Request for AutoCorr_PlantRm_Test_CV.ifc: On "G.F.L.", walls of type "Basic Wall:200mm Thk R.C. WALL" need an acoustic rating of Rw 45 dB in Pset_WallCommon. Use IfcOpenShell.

First a look at what the model holds.

```python
import ifcopenshell
import ifcopenshell.util.element

model = ifcopenshell.open("AutoCorr_PlantRm_Test_CV.ifc")
print(model.schema)
storey = next(s for s in model.by_type("IfcBuildingStorey") if s.Name == "G.F.L.")
walls = [e for e in ifcopenshell.util.element.get_decomposition(storey) if e.is_a("IfcWall")]
seen = {}
for e in walls:
    element_type = ifcopenshell.util.element.get_type(e)
    key = (element_type.Name if element_type != e and element_type else None, ifcopenshell.util.element.get_pset(e, "Pset_WallCommon", "AcousticRating"))
    seen[key] = seen.get(key, 0) + 1
for (name, value), count in sorted(seen.items(), key=str):
    print(count, "x", name, "|", value)
```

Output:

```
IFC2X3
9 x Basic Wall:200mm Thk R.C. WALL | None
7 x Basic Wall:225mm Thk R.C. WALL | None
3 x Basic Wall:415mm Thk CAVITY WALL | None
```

```python
import ifcopenshell
import ifcopenshell.api.pset
import ifcopenshell.util.element

model = ifcopenshell.open("AutoCorr_PlantRm_Test_CV.ifc")

storey = next(s for s in model.by_type("IfcBuildingStorey") if s.Name == "G.F.L.")
walls = [e for e in ifcopenshell.util.element.get_decomposition(storey) if e.is_a("IfcWall")]

count = 0
for e in walls:
    element_type = ifcopenshell.util.element.get_type(e)
    if element_type in (None, e) or element_type.Name != "Basic Wall:200mm Thk R.C. WALL":
        continue
    # add_pset returns the element's existing set when there is one.
    pset = ifcopenshell.api.pset.add_pset(model, product=e, name="Pset_WallCommon")
    ifcopenshell.api.pset.edit_pset(model, pset=pset, properties={"AcousticRating": "Rw 45 dB"})
    count += 1

print(count, "walls updated")

model.write("AutoCorr_PlantRm_Test_CV_edited.ifc")
```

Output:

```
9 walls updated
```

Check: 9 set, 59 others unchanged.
